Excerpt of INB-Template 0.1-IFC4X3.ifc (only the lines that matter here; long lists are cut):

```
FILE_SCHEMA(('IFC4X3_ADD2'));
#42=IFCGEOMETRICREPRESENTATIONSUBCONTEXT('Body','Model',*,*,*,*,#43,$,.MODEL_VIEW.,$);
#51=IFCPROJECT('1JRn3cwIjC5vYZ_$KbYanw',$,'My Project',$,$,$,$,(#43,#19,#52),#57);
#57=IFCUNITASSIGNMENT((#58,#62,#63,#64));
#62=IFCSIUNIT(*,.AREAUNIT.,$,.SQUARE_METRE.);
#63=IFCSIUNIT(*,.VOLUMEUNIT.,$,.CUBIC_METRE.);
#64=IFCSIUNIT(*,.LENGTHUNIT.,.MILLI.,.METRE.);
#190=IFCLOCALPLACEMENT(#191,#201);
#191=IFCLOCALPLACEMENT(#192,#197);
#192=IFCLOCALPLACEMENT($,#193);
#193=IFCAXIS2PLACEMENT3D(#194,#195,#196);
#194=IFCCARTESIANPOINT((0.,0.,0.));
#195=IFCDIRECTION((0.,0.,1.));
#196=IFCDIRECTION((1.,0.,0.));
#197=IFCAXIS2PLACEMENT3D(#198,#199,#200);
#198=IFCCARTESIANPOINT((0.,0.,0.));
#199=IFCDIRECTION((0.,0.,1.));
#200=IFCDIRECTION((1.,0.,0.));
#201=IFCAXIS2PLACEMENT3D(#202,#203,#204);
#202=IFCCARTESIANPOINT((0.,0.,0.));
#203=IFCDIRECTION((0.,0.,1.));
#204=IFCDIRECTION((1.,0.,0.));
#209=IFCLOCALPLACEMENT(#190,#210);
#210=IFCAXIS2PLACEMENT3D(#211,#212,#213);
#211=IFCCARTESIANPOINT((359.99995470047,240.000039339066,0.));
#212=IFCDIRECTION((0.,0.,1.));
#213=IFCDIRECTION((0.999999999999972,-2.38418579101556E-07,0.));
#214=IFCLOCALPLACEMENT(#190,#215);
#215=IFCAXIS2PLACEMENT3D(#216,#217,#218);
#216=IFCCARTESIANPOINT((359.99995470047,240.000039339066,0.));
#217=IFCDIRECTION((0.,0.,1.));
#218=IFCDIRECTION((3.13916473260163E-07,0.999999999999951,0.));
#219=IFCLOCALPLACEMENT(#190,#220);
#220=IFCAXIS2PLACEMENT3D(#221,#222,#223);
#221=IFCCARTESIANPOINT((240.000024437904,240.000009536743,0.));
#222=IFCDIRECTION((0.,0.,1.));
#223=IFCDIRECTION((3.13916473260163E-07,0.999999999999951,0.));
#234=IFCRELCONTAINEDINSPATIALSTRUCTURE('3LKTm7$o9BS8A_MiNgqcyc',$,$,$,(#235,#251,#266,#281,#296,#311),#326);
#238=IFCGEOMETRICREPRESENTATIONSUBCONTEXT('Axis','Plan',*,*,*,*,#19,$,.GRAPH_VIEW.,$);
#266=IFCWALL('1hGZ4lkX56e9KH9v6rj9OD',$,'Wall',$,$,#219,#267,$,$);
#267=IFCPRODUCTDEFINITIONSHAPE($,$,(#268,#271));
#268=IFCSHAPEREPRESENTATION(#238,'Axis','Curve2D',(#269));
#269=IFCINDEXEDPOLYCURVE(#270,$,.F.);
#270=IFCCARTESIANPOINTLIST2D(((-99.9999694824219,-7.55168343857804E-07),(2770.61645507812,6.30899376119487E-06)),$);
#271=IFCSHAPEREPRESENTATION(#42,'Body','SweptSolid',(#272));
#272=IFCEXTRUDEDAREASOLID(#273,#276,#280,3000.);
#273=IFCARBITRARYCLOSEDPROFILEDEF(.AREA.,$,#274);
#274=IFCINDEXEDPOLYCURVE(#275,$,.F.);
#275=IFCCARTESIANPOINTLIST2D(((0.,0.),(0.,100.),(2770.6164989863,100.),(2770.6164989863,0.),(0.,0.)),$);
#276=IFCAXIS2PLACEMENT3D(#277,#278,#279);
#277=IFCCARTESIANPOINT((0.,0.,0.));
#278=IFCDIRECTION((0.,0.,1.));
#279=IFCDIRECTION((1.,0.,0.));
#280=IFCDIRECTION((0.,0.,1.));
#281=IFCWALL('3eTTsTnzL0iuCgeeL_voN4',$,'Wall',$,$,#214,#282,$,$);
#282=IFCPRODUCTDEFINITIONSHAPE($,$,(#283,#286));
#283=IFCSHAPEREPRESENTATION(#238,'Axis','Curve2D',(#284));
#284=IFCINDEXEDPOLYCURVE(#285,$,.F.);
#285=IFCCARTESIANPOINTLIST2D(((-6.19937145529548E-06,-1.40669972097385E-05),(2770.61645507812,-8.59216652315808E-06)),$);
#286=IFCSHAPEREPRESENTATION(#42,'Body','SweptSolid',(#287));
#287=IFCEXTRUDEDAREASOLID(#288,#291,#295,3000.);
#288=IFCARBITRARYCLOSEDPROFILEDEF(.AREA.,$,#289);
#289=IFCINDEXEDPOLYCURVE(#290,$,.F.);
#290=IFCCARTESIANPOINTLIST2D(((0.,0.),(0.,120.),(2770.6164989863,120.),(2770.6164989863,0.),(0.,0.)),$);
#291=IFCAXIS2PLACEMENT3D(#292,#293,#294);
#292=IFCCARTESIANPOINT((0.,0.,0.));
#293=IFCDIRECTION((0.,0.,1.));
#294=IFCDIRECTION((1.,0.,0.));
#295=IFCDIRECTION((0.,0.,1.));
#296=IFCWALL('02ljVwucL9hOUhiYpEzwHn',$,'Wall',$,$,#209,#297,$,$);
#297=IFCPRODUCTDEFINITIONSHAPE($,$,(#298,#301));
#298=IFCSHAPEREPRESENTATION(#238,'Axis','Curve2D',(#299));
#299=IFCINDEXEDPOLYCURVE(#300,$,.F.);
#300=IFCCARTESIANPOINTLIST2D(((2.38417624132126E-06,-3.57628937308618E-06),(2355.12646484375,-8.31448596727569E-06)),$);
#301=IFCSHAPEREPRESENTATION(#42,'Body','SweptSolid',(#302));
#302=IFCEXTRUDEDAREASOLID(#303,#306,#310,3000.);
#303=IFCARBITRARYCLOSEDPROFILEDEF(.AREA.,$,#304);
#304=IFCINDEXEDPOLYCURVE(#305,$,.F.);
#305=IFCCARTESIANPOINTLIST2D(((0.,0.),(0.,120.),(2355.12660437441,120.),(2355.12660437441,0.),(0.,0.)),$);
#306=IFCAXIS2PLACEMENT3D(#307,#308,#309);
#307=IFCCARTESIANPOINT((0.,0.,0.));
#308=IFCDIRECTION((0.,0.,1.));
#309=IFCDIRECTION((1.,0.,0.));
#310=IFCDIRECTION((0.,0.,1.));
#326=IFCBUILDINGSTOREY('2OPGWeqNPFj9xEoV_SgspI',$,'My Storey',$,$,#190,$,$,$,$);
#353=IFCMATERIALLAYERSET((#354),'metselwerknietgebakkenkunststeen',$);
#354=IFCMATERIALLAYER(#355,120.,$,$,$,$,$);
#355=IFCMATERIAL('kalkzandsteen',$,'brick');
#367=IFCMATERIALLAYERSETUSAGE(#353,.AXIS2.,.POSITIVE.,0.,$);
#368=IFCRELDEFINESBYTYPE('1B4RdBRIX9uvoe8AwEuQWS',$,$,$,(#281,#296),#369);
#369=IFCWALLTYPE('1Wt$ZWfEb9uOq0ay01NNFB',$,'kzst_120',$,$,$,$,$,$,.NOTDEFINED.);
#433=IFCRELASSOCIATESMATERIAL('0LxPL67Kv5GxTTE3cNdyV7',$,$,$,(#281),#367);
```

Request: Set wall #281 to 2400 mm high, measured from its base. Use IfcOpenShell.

```python
import ifcopenshell
import ifcopenshell.geom
import ifcopenshell.util.representation
import ifcopenshell.util.shape
import ifcopenshell.util.unit

model = ifcopenshell.open("INB-Template 0.1-IFC4X3.ifc")
unit_scale = ifcopenshell.util.unit.calculate_unit_scale(model)
settings = ifcopenshell.geom.settings()


def volume(element):
    """Net volume in cubic metres, openings subtracted."""
    shape = ifcopenshell.geom.create_shape(settings, element)
    return ifcopenshell.util.shape.get_volume(shape.geometry)


wall = model.by_guid("3eTTsTnzL0iuCgeeL_voN4")
before = volume(wall)

body = ifcopenshell.util.representation.get_representation(wall, "Model", "Body")
solid = body.Items[0]
old_height = solid.Depth
solid.Depth = 2.4 / unit_scale
after = volume(wall)

print(f"height {old_height:g} -> {solid.Depth:g}, volume {before:.3f} -> {after:.3f} m3")

model.write("INB-Template 0.1-IFC4X3_v2.ifc")
```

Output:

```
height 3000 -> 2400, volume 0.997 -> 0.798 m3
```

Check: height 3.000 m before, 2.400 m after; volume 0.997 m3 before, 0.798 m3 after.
